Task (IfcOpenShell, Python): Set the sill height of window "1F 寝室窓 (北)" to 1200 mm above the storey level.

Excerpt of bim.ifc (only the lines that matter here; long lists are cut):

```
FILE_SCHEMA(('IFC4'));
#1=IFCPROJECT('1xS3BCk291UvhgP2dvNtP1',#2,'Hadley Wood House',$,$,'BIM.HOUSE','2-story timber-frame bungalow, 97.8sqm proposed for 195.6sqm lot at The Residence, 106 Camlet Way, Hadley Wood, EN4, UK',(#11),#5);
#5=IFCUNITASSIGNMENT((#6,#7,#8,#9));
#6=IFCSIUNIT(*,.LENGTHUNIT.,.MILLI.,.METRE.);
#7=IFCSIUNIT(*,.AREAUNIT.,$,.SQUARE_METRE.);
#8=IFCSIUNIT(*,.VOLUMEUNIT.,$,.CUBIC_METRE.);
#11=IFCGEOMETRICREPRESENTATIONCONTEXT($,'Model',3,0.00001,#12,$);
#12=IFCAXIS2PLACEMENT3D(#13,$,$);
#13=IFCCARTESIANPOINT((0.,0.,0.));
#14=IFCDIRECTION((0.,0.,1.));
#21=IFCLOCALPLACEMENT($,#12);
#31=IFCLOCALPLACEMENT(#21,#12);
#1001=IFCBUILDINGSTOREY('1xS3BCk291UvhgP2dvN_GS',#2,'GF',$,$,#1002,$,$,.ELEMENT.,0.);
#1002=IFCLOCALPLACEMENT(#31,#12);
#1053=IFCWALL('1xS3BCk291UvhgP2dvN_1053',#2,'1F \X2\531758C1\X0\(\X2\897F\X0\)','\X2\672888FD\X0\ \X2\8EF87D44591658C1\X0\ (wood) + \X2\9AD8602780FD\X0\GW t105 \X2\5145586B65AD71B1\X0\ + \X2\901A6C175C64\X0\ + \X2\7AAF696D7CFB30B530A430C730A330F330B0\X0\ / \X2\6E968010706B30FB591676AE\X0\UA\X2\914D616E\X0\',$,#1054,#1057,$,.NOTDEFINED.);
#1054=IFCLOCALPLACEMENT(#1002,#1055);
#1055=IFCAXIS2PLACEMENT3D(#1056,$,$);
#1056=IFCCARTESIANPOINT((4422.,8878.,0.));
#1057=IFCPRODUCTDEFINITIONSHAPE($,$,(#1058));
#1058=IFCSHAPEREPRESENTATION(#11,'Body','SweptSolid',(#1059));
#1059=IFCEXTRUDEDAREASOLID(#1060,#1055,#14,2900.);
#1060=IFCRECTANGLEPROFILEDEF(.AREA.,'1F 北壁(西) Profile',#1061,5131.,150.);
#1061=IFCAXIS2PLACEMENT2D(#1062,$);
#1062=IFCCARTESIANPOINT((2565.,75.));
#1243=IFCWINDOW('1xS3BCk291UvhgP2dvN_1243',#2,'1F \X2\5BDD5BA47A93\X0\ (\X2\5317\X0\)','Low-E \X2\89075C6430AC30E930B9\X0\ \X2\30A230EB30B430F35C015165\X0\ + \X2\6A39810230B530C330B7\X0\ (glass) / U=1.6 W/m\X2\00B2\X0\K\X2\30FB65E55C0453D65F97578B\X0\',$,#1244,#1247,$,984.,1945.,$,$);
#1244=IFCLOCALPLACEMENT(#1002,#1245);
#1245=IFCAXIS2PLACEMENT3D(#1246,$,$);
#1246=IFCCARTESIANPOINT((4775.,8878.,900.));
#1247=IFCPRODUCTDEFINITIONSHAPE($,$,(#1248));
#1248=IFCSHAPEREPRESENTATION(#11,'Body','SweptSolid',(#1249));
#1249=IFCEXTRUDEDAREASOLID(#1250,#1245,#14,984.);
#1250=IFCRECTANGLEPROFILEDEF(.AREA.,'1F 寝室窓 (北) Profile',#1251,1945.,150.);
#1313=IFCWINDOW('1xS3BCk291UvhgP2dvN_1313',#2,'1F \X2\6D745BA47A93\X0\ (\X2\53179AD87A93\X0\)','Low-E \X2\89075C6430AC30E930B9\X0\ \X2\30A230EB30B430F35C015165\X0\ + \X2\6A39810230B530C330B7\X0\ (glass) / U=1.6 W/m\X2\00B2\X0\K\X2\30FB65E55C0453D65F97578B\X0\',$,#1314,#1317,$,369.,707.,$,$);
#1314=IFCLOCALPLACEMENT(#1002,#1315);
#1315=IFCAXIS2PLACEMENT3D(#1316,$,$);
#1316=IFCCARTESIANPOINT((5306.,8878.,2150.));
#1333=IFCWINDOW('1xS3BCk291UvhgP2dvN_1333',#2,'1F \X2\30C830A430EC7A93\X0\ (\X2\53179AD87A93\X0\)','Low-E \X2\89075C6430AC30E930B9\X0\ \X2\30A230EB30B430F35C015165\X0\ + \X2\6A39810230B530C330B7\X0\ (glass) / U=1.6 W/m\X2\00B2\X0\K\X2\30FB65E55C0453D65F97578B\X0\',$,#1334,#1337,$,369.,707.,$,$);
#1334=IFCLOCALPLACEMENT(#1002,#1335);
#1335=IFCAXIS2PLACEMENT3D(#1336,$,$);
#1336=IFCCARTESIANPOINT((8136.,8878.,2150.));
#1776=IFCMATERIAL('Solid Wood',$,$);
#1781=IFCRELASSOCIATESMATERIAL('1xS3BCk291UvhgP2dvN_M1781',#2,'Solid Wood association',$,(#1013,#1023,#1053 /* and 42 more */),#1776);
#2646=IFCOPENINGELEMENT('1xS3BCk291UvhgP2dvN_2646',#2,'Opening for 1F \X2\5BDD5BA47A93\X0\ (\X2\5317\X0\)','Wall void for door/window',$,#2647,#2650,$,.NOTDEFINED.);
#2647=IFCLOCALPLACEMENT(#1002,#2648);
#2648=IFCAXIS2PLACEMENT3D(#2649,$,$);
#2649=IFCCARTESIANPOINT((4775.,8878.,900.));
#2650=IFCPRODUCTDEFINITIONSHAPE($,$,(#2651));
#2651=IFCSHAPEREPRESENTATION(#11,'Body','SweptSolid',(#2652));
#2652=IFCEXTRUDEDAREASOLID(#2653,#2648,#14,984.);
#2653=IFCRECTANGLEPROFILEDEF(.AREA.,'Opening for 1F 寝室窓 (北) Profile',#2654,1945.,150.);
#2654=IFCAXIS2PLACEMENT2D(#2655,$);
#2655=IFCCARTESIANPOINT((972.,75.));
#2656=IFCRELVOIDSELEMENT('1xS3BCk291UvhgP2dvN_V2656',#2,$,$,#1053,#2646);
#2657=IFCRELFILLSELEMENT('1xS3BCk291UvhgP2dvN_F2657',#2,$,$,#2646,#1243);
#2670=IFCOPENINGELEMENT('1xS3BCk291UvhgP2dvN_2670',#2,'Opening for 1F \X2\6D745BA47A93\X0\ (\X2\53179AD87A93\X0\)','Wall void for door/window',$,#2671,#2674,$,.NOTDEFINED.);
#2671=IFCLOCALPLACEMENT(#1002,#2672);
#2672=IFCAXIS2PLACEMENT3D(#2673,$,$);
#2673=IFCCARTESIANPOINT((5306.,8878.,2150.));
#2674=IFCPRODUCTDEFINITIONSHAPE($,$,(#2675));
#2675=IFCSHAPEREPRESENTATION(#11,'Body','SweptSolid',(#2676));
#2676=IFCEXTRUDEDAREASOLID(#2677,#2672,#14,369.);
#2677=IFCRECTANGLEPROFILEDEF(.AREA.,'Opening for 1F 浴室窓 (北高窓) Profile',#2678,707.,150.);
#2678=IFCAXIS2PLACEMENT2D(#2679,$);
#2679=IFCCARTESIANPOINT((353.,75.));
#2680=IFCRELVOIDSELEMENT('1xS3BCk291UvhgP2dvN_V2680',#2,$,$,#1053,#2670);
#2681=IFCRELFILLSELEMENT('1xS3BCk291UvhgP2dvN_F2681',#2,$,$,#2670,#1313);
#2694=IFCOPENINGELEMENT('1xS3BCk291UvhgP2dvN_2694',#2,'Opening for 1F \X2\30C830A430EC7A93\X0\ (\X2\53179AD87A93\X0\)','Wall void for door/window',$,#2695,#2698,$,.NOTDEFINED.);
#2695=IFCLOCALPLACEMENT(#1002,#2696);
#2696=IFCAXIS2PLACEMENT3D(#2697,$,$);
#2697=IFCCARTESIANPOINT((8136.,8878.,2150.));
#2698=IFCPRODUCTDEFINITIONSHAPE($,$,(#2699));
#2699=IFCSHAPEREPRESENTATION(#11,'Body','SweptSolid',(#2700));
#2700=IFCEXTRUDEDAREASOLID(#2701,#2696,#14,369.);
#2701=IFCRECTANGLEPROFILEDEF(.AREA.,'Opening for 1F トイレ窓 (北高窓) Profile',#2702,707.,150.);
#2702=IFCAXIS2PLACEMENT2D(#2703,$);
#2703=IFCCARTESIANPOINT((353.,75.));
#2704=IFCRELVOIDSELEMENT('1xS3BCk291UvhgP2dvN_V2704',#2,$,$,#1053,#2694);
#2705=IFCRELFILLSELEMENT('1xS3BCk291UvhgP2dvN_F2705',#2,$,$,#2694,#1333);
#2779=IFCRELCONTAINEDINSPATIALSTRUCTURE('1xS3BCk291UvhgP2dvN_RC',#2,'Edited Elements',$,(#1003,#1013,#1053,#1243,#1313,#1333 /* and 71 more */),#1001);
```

```python
import numpy as np
import ifcopenshell
import ifcopenshell.api.geometry
import ifcopenshell.geom
import ifcopenshell.util.element
import ifcopenshell.util.placement
import ifcopenshell.util.shape
import ifcopenshell.util.unit

model = ifcopenshell.open("bim.ifc")
unit_scale = ifcopenshell.util.unit.calculate_unit_scale(model)

window = model.by_guid("1xS3BCk291UvhgP2dvN_1243")
opening = window.FillsVoids[0].RelatingOpeningElement
storey = ifcopenshell.util.element.get_container(window, ifc_class="IfcBuildingStorey")
level = ifcopenshell.util.placement.get_local_placement(storey.ObjectPlacement)[2, 3]

# The opening's origin need not be at the sill, so measure its lowest point.
shape = ifcopenshell.geom.create_shape(ifcopenshell.geom.settings(), opening)
bottom = ifcopenshell.util.shape.get_shape_bottom_elevation(shape, shape.geometry) / unit_scale
dz = level + 1.2 / unit_scale - bottom

shift = np.array([0.0, 0.0, dz])
# The window is not placed relative to its opening, so move both.
for product in (opening, window):
    matrix = ifcopenshell.util.placement.get_local_placement(product.ObjectPlacement)
    matrix[:3, 3] += shift
    ifcopenshell.api.geometry.edit_object_placement(model, product=product, matrix=matrix, is_si=False)

print(f"moved by {dz * unit_scale:+.3f} m")

model.write("bim-out.ifc")
```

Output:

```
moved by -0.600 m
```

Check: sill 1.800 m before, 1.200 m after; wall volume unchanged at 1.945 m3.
